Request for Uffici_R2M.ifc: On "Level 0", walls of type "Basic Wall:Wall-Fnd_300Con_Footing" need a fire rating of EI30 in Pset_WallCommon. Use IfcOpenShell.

First a look at what the model holds.

```python
import ifcopenshell
import ifcopenshell.util.element

model = ifcopenshell.open("Uffici_R2M.ifc")
print(model.schema)
storey = next(s for s in model.by_type("IfcBuildingStorey") if s.Name == "Level 0")
walls = [e for e in ifcopenshell.util.element.get_decomposition(storey) if e.is_a("IfcWall")]
seen = {}
for e in walls:
    element_type = ifcopenshell.util.element.get_type(e)
    key = (element_type.Name if element_type != e and element_type else None, ifcopenshell.util.element.get_pset(e, "Pset_WallCommon", "FireRating"))
    seen[key] = seen.get(key, 0) + 1
for (name, value), count in sorted(seen.items(), key=str):
    print(count, "x", name, "|", value)
```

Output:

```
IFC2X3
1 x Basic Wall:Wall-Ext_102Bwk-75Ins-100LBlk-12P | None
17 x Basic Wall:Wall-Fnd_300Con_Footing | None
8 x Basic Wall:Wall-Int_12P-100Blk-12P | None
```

```python
import ifcopenshell
import ifcopenshell.api.pset
import ifcopenshell.util.element

model = ifcopenshell.open("Uffici_R2M.ifc")

storey = next(s for s in model.by_type("IfcBuildingStorey") if s.Name == "Level 0")
walls = [e for e in ifcopenshell.util.element.get_decomposition(storey) if e.is_a("IfcWall")]

count = 0
for e in walls:
    element_type = ifcopenshell.util.element.get_type(e)
    if element_type in (None, e) or element_type.Name != "Basic Wall:Wall-Fnd_300Con_Footing":
        continue
    # add_pset returns the element's existing set when there is one.
    pset = ifcopenshell.api.pset.add_pset(model, product=e, name="Pset_WallCommon")
    ifcopenshell.api.pset.edit_pset(model, pset=pset, properties={"FireRating": "EI30"})
    count += 1

print(count, "walls updated")

model.write("Uffici_R2M_edited.ifc")
```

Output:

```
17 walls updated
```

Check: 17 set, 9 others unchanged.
